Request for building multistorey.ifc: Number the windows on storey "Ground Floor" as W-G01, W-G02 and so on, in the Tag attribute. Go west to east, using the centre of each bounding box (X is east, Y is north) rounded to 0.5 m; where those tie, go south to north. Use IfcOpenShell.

First a look at what the model holds.

```python
import ifcopenshell
import ifcopenshell.util.element
import ifcopenshell.util.placement

model = ifcopenshell.open("building multistorey.ifc")
print(model.schema)
storey = next(s for s in model.by_type("IfcBuildingStorey") if s.Name == "Ground Floor")
windows = [e for e in ifcopenshell.util.element.get_decomposition(storey) if e.is_a("IfcWindow")]
for e in sorted(windows, key=lambda e: e.id()):
    origin = ifcopenshell.util.placement.get_local_placement(e.ObjectPlacement)[:3, 3]
    print(e.id(), e.Tag, e.Name, origin.round(2) + 0.0, sep=" | ")
```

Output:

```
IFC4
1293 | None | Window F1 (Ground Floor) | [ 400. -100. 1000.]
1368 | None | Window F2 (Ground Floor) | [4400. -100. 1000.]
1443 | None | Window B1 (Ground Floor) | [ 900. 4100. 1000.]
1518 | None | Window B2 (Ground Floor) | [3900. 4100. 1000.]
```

```python
import ifcopenshell
import ifcopenshell.geom
import ifcopenshell.util.element
import ifcopenshell.util.shape

model = ifcopenshell.open("building multistorey.ifc")
settings = ifcopenshell.geom.settings()
settings.set("use-world-coords", True)


def centre(element):
    shape = ifcopenshell.geom.create_shape(settings, element)
    return ifcopenshell.util.shape.get_bbox_centroid(shape.geometry)


storey = next(s for s in model.by_type("IfcBuildingStorey") if s.Name == "Ground Floor")
windows = [e for e in ifcopenshell.util.element.get_decomposition(storey) if e.is_a("IfcWindow")]

# Insertion points can sit at a corner or the storey origin, so sort by the geometry (in metres).
centres = {e: centre(e) for e in windows}
windows.sort(key=lambda e: (round(centres[e][0] / 0.5), centres[e][1]))

for i, e in enumerate(windows, start=1):
    number = f"W-G{i:02d}"
    e.Tag = number
    print(e.id(), number)

model.write("building multistorey_updated.ifc")
```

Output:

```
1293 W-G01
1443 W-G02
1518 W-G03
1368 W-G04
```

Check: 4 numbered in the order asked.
